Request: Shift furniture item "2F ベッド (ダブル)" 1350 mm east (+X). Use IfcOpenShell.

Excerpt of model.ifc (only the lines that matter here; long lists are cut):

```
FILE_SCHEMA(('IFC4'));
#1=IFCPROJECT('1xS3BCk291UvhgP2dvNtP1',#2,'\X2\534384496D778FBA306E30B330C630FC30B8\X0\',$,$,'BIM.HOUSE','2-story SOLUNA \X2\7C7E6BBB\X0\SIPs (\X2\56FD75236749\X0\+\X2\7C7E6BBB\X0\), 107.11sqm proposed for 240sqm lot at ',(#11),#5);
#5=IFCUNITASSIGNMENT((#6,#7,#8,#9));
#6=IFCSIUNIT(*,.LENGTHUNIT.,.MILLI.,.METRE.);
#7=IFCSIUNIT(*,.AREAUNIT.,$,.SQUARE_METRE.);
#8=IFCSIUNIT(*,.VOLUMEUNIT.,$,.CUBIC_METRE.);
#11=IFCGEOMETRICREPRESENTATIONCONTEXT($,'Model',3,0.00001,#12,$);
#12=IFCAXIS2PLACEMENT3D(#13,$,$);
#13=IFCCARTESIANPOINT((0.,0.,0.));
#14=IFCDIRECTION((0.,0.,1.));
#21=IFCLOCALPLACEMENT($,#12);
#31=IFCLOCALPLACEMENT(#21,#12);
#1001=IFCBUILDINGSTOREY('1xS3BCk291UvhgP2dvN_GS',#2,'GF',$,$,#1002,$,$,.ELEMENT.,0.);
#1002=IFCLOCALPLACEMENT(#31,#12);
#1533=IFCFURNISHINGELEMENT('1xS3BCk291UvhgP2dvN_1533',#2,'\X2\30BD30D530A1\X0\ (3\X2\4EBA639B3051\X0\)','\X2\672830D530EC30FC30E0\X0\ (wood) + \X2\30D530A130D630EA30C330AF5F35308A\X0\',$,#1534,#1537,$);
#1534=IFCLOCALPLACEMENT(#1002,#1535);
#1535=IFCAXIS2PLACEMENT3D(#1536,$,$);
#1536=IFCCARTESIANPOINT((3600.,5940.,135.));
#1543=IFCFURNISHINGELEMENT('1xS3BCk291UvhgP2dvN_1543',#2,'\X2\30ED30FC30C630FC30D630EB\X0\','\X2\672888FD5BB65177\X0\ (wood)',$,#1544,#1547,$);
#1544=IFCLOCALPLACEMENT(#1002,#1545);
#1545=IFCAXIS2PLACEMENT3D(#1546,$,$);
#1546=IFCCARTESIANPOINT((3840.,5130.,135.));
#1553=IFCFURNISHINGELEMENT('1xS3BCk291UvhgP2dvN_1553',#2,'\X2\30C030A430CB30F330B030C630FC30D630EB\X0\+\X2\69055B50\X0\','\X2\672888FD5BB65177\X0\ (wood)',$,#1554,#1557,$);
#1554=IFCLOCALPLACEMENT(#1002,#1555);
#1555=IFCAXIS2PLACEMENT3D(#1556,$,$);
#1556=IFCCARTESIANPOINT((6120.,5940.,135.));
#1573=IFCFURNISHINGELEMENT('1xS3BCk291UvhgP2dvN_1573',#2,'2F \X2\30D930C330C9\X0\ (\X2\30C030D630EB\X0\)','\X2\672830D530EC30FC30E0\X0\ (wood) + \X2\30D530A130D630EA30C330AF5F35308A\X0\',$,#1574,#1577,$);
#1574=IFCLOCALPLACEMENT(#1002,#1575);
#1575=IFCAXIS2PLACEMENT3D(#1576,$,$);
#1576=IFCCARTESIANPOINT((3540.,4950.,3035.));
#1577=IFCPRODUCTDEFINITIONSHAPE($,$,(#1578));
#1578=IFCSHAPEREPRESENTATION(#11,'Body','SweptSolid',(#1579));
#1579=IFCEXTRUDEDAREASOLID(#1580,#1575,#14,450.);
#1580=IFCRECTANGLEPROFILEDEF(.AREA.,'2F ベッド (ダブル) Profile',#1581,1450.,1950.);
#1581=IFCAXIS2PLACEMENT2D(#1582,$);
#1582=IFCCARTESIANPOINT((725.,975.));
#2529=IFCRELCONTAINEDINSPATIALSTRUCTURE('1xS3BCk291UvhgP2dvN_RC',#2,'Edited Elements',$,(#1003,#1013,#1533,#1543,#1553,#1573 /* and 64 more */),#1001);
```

```python
import ifcopenshell
import ifcopenshell.api.geometry
import ifcopenshell.util.placement
import ifcopenshell.util.unit

model = ifcopenshell.open("model.ifc")
unit_scale = ifcopenshell.util.unit.calculate_unit_scale(model)

item = model.by_id(1573)
matrix = ifcopenshell.util.placement.get_local_placement(item.ObjectPlacement)
matrix[0, 3] += 1.35 / unit_scale
ifcopenshell.api.geometry.edit_object_placement(model, product=item, matrix=matrix, is_si=False)

print(ifcopenshell.util.placement.get_local_placement(item.ObjectPlacement).round(3) + 0.0)

model.write("model_edited.ifc")
```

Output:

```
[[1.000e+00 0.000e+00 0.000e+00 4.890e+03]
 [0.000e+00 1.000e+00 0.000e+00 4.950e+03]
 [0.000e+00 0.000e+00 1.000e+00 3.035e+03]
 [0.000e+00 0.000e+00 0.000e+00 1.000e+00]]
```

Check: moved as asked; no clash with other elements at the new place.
